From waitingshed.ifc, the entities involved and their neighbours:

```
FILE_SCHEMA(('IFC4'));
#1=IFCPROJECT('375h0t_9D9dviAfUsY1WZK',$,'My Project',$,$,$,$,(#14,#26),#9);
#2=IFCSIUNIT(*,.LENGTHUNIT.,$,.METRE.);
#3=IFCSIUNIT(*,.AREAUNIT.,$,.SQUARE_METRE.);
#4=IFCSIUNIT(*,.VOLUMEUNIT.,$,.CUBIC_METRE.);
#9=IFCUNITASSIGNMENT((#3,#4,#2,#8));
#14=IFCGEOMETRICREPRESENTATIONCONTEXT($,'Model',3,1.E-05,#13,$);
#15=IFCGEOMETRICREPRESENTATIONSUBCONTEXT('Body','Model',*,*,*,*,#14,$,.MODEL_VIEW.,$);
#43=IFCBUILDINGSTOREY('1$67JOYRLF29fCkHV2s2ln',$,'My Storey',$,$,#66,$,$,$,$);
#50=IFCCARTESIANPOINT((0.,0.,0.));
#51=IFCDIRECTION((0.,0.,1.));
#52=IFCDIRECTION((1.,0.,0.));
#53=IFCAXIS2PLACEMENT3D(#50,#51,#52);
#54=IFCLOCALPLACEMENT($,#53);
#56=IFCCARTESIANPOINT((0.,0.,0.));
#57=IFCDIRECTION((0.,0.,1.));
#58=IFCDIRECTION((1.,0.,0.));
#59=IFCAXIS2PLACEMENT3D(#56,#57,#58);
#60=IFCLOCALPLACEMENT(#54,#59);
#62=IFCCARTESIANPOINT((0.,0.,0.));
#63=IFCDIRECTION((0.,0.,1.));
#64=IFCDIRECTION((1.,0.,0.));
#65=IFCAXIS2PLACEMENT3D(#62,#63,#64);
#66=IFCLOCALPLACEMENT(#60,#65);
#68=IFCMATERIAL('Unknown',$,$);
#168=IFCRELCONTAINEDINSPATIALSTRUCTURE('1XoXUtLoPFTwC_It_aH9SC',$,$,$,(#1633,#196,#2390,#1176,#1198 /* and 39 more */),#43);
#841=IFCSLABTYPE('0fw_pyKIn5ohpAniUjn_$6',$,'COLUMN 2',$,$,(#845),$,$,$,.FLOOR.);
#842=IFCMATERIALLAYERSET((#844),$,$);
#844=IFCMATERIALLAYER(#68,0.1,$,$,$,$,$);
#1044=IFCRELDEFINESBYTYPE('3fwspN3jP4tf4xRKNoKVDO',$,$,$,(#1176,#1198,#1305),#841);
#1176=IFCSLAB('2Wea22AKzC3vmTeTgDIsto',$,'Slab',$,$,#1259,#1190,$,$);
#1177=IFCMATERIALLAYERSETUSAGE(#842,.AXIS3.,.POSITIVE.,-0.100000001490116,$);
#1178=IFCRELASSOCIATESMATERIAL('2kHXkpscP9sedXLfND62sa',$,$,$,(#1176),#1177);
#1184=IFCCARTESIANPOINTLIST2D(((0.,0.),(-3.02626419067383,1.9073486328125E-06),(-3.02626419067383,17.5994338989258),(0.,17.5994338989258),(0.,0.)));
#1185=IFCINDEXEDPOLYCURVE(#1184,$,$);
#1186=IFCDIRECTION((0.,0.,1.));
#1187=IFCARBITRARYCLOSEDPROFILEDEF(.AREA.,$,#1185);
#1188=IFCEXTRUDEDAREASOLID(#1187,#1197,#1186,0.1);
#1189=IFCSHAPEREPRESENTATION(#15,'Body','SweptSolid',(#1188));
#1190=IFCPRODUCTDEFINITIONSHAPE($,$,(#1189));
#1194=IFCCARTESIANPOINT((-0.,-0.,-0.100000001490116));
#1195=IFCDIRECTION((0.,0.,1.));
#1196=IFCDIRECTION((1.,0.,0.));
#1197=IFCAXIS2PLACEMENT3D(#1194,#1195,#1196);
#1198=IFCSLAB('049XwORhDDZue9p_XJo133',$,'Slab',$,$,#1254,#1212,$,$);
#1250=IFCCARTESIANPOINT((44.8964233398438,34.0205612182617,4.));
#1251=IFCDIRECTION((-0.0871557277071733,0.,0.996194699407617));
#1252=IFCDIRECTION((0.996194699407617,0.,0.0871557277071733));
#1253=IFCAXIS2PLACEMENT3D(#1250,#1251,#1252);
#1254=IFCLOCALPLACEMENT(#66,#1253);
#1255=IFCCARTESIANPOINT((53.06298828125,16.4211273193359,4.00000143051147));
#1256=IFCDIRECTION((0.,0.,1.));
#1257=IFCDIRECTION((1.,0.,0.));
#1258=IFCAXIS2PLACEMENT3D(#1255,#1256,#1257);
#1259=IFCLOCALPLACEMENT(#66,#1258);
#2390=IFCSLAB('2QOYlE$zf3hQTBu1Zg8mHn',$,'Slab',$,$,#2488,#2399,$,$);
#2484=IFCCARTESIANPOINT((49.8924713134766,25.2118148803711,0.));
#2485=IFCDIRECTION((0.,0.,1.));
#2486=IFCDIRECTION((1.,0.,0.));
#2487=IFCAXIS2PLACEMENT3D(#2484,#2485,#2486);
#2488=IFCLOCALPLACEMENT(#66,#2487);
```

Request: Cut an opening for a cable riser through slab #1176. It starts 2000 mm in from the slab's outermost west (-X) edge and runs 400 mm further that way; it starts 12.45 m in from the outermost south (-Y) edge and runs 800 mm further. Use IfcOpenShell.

```python
import numpy as np
import ifcopenshell
import ifcopenshell.api.feature
import ifcopenshell.api.geometry
import ifcopenshell.api.root
import ifcopenshell.geom
import ifcopenshell.util.placement
import ifcopenshell.util.representation
import ifcopenshell.util.shape
import ifcopenshell.util.unit

model = ifcopenshell.open("waitingshed.ifc")
unit_scale = ifcopenshell.util.unit.calculate_unit_scale(model)
settings = ifcopenshell.geom.settings()


def volume(element):
    """Net volume in cubic metres, openings subtracted."""
    shape = ifcopenshell.geom.create_shape(settings, element)
    return ifcopenshell.util.shape.get_volume(shape.geometry)


slab = model.by_guid("2Wea22AKzC3vmTeTgDIsto")
before = volume(slab)

# Extent in the slab's own axes, in metres. The edges named are its -X and -Y sides.
slab_shape = ifcopenshell.geom.create_shape(settings, slab)
vertices = ifcopenshell.util.shape.get_vertices(slab_shape.geometry)
x_min, y_min, bottom = vertices.min(axis=0)
top = vertices[:, 2].max()

opening = ifcopenshell.api.root.create_entity(model, ifc_class="IfcOpeningElement", name="Cable riser opening", predefined_type="OPENING")
context = ifcopenshell.util.representation.get_context(model, "Model", "Body", "MODEL_VIEW")
width, depth = 0.4, 0.8
outline = [(0.0, 0.0), (width, 0.0), (width, depth), (0.0, depth), (0.0, 0.0)]
# Overshoot both faces by 50 mm so the cut is clean.
shape = ifcopenshell.api.geometry.add_slab_representation(
    model, context=context, depth=top - bottom + 0.1, polyline=outline
)
ifcopenshell.api.geometry.assign_representation(model, product=opening, representation=shape)

matrix = ifcopenshell.util.placement.get_local_placement(slab.ObjectPlacement)
matrix[:, 3] = matrix @ np.append(np.array([x_min + 2, y_min + 12.45, bottom - 0.05]) / unit_scale, 1.0)
ifcopenshell.api.geometry.edit_object_placement(model, product=opening, matrix=matrix, is_si=False)
ifcopenshell.api.feature.add_feature(model, feature=opening, element=slab)

after = volume(slab)

print(f"slab volume {before:.3f} -> {after:.3f} m3")

model.write("waitingshed_rev.ifc")
```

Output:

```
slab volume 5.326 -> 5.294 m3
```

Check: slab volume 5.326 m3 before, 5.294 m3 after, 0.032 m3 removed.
